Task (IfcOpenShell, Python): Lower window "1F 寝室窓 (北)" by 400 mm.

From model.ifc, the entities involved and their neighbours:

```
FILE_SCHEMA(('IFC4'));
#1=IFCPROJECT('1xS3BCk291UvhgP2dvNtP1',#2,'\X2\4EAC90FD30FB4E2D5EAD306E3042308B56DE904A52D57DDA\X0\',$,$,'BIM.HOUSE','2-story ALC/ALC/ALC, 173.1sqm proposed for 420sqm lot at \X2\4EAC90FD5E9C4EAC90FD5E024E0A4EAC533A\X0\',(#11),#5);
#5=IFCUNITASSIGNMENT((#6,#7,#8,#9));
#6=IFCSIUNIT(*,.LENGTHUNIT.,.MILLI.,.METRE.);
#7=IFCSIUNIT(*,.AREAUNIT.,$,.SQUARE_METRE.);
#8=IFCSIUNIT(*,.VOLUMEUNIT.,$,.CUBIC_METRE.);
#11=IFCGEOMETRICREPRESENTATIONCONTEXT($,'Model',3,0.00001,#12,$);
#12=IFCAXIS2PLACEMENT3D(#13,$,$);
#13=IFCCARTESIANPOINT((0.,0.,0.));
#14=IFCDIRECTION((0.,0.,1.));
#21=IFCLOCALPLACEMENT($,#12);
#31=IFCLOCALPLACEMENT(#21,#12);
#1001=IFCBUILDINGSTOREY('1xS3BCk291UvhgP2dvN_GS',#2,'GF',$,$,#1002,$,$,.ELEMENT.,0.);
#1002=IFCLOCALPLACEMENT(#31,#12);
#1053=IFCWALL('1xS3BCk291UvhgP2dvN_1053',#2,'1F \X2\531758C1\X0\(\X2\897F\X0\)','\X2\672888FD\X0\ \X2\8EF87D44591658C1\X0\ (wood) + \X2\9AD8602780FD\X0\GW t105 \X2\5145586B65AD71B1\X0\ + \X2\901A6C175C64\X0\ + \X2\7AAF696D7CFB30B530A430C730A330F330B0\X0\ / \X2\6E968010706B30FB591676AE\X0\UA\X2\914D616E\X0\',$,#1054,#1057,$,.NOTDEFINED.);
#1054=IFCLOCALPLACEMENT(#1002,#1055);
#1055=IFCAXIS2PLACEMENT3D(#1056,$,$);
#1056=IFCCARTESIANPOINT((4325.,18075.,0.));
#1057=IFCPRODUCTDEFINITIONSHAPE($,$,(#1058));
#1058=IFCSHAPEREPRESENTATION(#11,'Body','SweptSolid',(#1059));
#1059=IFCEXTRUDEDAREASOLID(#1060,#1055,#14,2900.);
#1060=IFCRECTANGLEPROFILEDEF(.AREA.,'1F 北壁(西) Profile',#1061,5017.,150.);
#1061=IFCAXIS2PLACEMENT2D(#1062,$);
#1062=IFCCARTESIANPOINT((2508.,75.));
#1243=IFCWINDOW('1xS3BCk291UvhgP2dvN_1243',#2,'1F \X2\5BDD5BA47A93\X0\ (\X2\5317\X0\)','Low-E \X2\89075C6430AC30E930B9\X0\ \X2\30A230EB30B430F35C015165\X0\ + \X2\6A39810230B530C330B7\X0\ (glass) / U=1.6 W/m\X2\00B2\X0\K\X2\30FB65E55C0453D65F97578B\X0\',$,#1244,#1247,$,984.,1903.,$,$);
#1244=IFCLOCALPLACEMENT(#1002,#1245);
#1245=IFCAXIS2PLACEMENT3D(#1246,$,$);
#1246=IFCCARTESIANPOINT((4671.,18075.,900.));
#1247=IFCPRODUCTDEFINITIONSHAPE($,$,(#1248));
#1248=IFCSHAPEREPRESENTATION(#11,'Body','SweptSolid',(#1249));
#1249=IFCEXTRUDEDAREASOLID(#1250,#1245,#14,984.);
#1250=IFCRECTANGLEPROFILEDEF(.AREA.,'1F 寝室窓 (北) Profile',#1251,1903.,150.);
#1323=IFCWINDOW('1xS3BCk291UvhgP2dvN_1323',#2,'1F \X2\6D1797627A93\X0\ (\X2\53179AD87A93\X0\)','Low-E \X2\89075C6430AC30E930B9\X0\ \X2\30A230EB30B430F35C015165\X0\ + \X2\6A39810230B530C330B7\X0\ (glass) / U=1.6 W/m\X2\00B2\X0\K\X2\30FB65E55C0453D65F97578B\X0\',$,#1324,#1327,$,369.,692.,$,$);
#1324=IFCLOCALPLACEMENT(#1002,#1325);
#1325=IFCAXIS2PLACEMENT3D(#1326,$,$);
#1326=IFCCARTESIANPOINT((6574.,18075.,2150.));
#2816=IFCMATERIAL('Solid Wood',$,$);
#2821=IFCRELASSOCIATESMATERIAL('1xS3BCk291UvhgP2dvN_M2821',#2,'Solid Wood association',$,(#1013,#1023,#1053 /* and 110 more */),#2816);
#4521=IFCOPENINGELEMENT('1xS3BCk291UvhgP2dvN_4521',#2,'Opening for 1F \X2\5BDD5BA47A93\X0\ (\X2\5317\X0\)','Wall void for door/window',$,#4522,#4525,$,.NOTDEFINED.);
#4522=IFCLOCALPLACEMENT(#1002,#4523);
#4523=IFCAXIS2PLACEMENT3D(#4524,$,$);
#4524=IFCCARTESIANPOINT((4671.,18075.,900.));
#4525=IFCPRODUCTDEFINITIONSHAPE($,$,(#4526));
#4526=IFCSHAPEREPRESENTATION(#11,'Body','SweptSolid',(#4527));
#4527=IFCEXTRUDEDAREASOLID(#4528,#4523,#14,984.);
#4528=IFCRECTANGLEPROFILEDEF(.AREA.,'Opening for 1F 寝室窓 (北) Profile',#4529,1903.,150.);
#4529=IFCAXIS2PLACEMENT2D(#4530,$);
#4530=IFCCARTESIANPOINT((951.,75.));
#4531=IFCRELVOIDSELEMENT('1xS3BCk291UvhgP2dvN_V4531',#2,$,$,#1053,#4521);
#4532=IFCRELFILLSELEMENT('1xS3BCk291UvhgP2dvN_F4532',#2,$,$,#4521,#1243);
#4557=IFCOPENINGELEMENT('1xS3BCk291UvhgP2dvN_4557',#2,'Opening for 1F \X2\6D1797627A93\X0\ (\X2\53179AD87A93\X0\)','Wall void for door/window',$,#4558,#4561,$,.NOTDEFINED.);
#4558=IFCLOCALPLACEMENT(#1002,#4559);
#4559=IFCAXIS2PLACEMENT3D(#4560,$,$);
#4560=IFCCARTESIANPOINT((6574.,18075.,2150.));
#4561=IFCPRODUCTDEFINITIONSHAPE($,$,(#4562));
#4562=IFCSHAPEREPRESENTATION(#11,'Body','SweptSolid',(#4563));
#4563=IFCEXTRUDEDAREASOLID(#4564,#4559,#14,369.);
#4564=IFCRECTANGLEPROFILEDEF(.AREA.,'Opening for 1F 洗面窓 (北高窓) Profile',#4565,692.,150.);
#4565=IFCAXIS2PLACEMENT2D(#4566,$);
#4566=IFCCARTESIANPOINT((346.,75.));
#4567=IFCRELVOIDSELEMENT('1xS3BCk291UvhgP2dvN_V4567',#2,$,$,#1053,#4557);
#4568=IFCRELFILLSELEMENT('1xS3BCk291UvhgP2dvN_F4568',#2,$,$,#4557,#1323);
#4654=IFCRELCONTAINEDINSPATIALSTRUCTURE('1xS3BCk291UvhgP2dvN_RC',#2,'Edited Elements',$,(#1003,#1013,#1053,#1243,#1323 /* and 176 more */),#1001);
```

```python
import numpy as np
import ifcopenshell
import ifcopenshell.api.geometry
import ifcopenshell.util.placement
import ifcopenshell.util.unit

model = ifcopenshell.open("model.ifc")
unit_scale = ifcopenshell.util.unit.calculate_unit_scale(model)

window = model.by_id(1243)
opening = window.FillsVoids[0].RelatingOpeningElement
dz = -400.0

shift = np.array([0.0, 0.0, dz])
# The window is not placed relative to its opening, so move both.
for product in (opening, window):
    matrix = ifcopenshell.util.placement.get_local_placement(product.ObjectPlacement)
    matrix[:3, 3] += shift
    ifcopenshell.api.geometry.edit_object_placement(model, product=product, matrix=matrix, is_si=False)

print(f"moved by {dz * unit_scale:+.3f} m")

model.write("model_edited.ifc")
```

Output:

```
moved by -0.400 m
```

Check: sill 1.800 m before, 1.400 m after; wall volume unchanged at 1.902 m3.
